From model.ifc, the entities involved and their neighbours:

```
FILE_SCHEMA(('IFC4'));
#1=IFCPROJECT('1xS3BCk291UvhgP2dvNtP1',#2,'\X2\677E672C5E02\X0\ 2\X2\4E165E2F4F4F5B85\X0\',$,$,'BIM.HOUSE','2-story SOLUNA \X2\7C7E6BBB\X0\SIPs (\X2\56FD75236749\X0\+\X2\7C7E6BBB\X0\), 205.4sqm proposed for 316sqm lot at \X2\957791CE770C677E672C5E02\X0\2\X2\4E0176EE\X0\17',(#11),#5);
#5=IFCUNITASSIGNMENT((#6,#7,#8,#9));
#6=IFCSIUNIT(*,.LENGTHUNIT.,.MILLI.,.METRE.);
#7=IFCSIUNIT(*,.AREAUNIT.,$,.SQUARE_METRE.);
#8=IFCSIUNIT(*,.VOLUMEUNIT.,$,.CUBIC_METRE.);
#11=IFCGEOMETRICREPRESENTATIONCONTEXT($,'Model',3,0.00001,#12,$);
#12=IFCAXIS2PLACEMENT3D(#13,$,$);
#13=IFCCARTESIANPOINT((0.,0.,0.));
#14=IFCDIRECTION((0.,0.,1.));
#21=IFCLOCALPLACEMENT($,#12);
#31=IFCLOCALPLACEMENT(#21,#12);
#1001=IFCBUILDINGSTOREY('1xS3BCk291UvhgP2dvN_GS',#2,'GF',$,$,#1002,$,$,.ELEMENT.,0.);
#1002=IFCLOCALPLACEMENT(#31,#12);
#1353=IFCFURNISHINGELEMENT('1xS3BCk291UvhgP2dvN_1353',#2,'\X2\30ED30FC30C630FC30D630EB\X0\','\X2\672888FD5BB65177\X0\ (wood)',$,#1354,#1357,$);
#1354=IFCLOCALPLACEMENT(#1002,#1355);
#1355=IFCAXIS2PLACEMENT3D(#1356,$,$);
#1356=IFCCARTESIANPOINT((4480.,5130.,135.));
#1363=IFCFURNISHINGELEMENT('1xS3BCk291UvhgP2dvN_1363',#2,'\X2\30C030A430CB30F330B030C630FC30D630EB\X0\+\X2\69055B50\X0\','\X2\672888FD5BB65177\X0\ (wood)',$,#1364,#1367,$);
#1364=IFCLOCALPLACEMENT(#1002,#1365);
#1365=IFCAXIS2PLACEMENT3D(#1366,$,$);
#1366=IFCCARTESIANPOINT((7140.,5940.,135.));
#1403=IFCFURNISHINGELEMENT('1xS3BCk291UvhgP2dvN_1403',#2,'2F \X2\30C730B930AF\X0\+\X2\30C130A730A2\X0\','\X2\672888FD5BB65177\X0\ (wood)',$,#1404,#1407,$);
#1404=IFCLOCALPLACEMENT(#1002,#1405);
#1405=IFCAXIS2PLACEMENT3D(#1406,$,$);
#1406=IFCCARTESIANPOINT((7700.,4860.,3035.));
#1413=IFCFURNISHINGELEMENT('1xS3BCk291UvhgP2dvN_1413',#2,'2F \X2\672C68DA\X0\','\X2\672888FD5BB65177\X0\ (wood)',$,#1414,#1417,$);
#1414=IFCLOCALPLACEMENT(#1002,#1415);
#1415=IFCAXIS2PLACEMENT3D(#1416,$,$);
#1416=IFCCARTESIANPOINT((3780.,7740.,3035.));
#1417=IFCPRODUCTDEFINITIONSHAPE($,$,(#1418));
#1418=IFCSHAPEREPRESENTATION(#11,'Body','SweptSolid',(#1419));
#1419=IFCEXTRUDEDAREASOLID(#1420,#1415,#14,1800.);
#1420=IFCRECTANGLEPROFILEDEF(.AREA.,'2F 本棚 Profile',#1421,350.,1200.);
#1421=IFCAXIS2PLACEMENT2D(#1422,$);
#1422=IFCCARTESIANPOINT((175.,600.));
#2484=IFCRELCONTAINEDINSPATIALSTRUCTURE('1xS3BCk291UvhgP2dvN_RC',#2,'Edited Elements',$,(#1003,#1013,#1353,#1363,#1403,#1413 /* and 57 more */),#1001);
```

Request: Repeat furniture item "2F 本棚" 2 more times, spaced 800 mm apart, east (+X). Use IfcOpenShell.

```python
import numpy as np
import ifcopenshell
import ifcopenshell.api.geometry
import ifcopenshell.api.root
import ifcopenshell.util.element
import ifcopenshell.util.placement

model = ifcopenshell.open("model.ifc")


def reuse_history(source, copy):
    """copy_class also copies each property set's owner history, people and application; keep the originals."""
    for rel in copy.IsDefinedBy:
        if rel.is_a("IfcRelDefinesByProperties") and (history := rel.RelatingPropertyDefinition.OwnerHistory):
            rel.RelatingPropertyDefinition.OwnerHistory = source.OwnerHistory
            ifcopenshell.util.element.remove_deep2(model, history)


source = model.by_id(1413)
base = ifcopenshell.util.placement.get_local_placement(source.ObjectPlacement)
step = np.array([1.0, 0.0, 0.0]) * 800.0

for i in range(1, 3):
    copy = ifcopenshell.api.root.copy_class(model, product=source)
    copy.Representation = ifcopenshell.util.element.copy_deep(
        model, source.Representation, exclude=["IfcGeometricRepresentationContext", "IfcRepresentationMap"]
    )
    reuse_history(source, copy)
    matrix = base.copy()
    matrix[:3, 3] += i * step
    print("added at", matrix[:3, 3].round(3) + 0.0)
    ifcopenshell.api.geometry.edit_object_placement(model, product=copy, matrix=matrix, is_si=False)

model.write("model_edited.ifc")
```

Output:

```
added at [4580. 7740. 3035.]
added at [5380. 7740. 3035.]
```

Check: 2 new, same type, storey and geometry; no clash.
